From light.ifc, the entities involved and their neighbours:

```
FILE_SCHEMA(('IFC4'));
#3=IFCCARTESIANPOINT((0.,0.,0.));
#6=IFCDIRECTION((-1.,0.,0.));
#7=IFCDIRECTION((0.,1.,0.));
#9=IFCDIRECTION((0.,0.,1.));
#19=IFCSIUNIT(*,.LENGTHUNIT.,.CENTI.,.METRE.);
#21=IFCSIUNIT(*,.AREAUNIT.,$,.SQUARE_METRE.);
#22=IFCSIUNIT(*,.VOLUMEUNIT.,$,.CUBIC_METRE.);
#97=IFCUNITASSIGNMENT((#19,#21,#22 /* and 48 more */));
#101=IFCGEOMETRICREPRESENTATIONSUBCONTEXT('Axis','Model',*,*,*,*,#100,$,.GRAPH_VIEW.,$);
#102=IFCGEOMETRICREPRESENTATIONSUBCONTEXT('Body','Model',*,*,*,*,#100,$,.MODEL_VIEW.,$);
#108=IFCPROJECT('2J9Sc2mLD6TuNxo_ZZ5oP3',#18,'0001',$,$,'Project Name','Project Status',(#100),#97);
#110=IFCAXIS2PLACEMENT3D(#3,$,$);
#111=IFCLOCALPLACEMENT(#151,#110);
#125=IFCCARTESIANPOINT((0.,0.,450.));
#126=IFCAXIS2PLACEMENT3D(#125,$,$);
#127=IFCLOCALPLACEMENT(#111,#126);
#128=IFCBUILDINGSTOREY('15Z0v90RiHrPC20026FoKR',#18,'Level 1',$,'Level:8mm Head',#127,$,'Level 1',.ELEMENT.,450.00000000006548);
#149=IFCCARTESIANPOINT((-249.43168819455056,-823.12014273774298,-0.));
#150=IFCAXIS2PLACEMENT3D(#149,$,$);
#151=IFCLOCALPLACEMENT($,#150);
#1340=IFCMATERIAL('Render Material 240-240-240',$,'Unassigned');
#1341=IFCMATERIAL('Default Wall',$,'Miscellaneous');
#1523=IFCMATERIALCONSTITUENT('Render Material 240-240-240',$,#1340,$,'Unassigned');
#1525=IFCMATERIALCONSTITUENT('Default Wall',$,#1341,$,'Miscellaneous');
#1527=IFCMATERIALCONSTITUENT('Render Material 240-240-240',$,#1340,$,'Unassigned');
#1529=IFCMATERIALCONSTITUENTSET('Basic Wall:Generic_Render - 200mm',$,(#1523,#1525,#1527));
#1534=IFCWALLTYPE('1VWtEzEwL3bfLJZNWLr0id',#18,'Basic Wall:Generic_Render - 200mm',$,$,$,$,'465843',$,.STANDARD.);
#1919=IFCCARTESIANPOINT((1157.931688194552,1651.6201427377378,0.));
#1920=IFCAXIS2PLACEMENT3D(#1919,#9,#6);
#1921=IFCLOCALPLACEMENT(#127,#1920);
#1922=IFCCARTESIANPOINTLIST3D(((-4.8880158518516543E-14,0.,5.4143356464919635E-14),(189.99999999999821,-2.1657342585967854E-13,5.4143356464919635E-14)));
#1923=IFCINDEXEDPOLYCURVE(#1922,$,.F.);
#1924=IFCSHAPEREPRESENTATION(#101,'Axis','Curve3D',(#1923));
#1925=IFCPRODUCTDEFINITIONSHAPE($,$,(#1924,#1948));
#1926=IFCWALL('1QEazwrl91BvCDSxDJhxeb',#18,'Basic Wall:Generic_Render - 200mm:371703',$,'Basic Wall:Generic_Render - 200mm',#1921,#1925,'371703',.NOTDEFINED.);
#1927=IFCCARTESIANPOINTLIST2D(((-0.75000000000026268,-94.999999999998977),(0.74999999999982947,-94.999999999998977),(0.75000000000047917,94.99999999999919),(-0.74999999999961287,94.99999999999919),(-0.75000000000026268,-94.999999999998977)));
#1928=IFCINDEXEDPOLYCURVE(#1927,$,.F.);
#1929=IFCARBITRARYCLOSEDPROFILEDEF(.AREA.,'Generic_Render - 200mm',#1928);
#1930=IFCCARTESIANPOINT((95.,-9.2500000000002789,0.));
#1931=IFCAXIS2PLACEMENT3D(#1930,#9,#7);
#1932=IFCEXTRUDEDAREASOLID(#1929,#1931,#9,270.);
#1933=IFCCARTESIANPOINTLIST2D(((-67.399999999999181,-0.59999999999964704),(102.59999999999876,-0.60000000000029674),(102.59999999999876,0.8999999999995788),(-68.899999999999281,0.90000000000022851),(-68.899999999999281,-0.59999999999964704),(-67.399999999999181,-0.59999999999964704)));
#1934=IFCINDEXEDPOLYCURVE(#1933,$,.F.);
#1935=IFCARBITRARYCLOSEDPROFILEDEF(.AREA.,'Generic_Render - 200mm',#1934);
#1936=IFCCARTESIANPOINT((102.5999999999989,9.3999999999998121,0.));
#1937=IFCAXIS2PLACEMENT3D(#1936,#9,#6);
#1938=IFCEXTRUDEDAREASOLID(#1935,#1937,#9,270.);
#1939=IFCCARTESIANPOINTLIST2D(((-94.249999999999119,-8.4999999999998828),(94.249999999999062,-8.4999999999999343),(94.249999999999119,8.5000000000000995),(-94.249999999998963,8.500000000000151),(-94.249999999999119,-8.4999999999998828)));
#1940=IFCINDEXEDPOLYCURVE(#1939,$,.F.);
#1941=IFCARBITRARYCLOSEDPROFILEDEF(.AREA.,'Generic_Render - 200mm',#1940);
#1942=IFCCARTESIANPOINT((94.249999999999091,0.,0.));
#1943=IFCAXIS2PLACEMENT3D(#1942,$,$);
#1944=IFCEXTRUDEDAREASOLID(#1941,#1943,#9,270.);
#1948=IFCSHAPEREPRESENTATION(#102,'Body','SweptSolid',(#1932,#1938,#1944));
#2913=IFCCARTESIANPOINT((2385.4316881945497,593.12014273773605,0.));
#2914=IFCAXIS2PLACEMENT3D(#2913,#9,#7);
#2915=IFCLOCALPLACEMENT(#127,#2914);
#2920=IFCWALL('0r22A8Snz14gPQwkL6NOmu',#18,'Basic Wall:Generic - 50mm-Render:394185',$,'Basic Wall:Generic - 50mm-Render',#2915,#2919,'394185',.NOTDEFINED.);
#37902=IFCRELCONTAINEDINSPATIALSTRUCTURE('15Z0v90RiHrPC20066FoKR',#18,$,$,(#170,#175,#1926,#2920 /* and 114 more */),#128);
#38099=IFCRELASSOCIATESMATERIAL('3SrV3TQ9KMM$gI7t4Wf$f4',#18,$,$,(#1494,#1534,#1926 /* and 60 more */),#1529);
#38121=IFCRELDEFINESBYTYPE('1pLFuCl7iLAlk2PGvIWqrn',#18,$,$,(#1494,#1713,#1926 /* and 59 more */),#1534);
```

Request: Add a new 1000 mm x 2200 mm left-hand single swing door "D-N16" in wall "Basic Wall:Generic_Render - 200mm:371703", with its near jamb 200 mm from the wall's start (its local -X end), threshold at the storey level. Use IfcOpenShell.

```python
import numpy as np
import ifcopenshell
import ifcopenshell.api.feature
import ifcopenshell.api.geometry
import ifcopenshell.api.root
import ifcopenshell.api.spatial
import ifcopenshell.geom
import ifcopenshell.util.element
import ifcopenshell.util.placement
import ifcopenshell.util.representation
import ifcopenshell.util.shape
import ifcopenshell.util.unit

model = ifcopenshell.open("light.ifc")
unit_scale = ifcopenshell.util.unit.calculate_unit_scale(model)
settings = ifcopenshell.geom.settings()


def volume(element):
    """Net volume in cubic metres, openings subtracted."""
    shape = ifcopenshell.geom.create_shape(settings, element)
    return ifcopenshell.util.shape.get_volume(shape.geometry)


wall = model.by_id(1926)
storey = ifcopenshell.util.element.get_container(wall, ifc_class="IfcBuildingStorey")
context = ifcopenshell.util.representation.get_context(model, "Model", "Body", "MODEL_VIEW")
before = volume(wall)

width, height, from_end, sill = 1, 2.2, 0.2, 0.0  # metres

# The wall runs along its own X axis, and the end named is its -X end.
wall_shape = ifcopenshell.geom.create_shape(settings, wall)
x, y, z = ifcopenshell.util.shape.get_vertices(wall_shape.geometry).T
start = x.min() + from_end
face, thickness = float(y.min()), float(y.max() - y.min())
wall_matrix = ifcopenshell.util.placement.get_local_placement(wall.ObjectPlacement)
level = ifcopenshell.util.placement.get_local_placement(storey.ObjectPlacement)[2, 3]


def in_wall(x, y):
    """Placement at x, y metres in the wall's axes, at sill height."""
    matrix = wall_matrix.copy()
    matrix[:, 3] = wall_matrix @ np.array([x / unit_scale, y / unit_scale, 0.0, 1.0])
    matrix[2, 3] = level + sill / unit_scale
    return matrix


# Opening: a box that overshoots both wall faces by 50 mm.
opening = ifcopenshell.api.root.create_entity(model, ifc_class="IfcOpeningElement", predefined_type="OPENING")
box = ifcopenshell.api.geometry.add_wall_representation(
    model, context=context, length=width, height=height, thickness=thickness + 0.1
)
ifcopenshell.api.geometry.assign_representation(model, product=opening, representation=box)
ifcopenshell.api.geometry.edit_object_placement(model, product=opening, matrix=in_wall(start, face - 0.05), is_si=False)
ifcopenshell.api.feature.add_feature(model, feature=opening, element=wall)

door = ifcopenshell.api.root.create_entity(model, ifc_class="IfcDoor", name="D-N16", predefined_type="DOOR")
door.OverallWidth, door.OverallHeight = width / unit_scale, height / unit_scale
door.OperationType = "SINGLE_SWING_LEFT"
body = ifcopenshell.api.geometry.add_door_representation(
    model,
    context=context,
    overall_width=door.OverallWidth,
    overall_height=door.OverallHeight,
    operation_type="SINGLE_SWING_LEFT",
    lining_properties={"LiningDepth": thickness / unit_scale, "ThresholdDepth": thickness / unit_scale},
)
ifcopenshell.api.geometry.assign_representation(model, product=door, representation=body)
ifcopenshell.api.spatial.assign_container(model, products=[door], relating_structure=storey)
ifcopenshell.api.feature.add_filling(model, opening=opening, element=door)

# The lining spans the wall, so the door starts at the wall face.
ifcopenshell.api.geometry.edit_object_placement(model, product=door, matrix=in_wall(start, face), is_si=False)

after = volume(wall)

print(f"wall volume {before:.3f} -> {after:.3f} m3")

model.write("light-out.ifc")
```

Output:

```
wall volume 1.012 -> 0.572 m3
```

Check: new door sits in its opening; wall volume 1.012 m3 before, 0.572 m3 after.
